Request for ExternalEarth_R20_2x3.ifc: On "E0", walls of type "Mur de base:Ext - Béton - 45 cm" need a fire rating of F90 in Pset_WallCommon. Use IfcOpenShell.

First a look at what the model holds.

```python
import ifcopenshell
import ifcopenshell.util.element

model = ifcopenshell.open("ExternalEarth_R20_2x3.ifc")
print(model.schema)
storey = next(s for s in model.by_type("IfcBuildingStorey") if s.Name == "E0")
walls = [e for e in ifcopenshell.util.element.get_decomposition(storey) if e.is_a("IfcWall")]
seen = {}
for e in walls:
    element_type = ifcopenshell.util.element.get_type(e)
    key = (element_type.Name if element_type != e and element_type else None, ifcopenshell.util.element.get_pset(e, "Pset_WallCommon", "FireRating"))
    seen[key] = seen.get(key, 0) + 1
for (name, value), count in sorted(seen.items(), key=str):
    print(count, "x", name, "|", value)
```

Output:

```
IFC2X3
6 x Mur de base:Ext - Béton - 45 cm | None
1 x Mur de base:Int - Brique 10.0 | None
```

```python
import ifcopenshell
import ifcopenshell.api.pset
import ifcopenshell.util.element

model = ifcopenshell.open("ExternalEarth_R20_2x3.ifc")

storey = next(s for s in model.by_type("IfcBuildingStorey") if s.Name == "E0")
walls = [e for e in ifcopenshell.util.element.get_decomposition(storey) if e.is_a("IfcWall")]

count = 0
for e in walls:
    element_type = ifcopenshell.util.element.get_type(e)
    if element_type in (None, e) or element_type.Name != "Mur de base:Ext - Béton - 45 cm":
        continue
    # add_pset returns the element's existing set when there is one.
    pset = ifcopenshell.api.pset.add_pset(model, product=e, name="Pset_WallCommon")
    ifcopenshell.api.pset.edit_pset(model, pset=pset, properties={"FireRating": "F90"})
    count += 1

print(count, "walls updated")

model.write("ExternalEarth_R20_2x3-out.ifc")
```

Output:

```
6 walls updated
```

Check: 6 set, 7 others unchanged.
